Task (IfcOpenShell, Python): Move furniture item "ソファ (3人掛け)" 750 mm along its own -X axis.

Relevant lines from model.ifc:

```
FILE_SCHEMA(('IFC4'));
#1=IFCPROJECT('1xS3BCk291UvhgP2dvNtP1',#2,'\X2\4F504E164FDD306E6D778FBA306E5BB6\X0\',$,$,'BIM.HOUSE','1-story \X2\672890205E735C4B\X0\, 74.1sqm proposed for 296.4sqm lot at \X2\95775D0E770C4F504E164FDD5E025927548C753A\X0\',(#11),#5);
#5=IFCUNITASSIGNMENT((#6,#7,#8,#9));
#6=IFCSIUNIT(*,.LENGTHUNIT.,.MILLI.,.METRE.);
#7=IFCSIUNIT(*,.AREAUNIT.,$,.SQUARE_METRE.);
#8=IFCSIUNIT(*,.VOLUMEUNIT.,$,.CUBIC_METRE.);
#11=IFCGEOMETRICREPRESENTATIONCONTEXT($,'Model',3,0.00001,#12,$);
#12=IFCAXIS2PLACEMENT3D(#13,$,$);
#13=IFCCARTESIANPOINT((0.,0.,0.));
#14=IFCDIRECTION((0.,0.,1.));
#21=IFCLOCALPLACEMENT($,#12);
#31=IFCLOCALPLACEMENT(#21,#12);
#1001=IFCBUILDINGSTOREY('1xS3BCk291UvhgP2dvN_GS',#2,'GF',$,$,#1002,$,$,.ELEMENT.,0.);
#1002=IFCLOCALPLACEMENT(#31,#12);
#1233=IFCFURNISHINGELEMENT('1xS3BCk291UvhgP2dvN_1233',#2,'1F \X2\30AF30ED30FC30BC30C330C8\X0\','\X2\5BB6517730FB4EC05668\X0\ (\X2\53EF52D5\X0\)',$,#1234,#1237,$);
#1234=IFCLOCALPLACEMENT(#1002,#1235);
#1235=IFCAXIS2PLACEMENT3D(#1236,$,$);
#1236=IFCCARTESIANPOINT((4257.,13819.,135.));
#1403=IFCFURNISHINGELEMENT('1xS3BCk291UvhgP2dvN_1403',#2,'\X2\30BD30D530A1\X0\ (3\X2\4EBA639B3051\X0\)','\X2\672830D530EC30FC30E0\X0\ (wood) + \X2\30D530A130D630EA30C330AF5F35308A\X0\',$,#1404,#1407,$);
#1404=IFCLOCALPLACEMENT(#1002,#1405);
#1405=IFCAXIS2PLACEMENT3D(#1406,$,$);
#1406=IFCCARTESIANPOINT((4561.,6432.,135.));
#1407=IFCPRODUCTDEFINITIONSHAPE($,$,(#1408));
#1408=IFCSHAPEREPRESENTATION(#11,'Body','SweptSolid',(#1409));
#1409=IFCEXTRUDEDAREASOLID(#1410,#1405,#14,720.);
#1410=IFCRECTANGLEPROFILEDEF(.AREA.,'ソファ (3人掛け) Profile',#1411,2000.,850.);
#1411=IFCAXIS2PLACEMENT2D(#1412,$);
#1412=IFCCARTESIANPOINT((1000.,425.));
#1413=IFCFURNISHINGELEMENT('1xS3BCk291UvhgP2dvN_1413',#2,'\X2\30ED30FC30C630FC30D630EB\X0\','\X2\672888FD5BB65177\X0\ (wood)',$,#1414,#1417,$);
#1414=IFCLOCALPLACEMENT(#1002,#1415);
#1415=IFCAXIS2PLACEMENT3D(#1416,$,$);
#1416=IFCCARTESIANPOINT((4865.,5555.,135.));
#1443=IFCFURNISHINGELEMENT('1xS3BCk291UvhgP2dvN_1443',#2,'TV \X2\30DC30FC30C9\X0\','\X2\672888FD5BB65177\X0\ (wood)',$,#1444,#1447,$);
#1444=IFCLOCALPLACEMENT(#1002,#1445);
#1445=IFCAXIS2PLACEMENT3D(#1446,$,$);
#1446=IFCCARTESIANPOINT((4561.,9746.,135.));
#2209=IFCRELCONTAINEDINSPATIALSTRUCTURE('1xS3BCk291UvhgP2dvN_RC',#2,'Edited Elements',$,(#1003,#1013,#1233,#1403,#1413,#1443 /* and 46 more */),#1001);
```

```python
import ifcopenshell
import ifcopenshell.api.geometry
import ifcopenshell.util.placement

model = ifcopenshell.open("model.ifc")

item = model.by_guid("1xS3BCk291UvhgP2dvN_1403")
matrix = ifcopenshell.util.placement.get_local_placement(item.ObjectPlacement)
matrix[:3, 3] -= matrix[:3, 0] * 750.0
ifcopenshell.api.geometry.edit_object_placement(model, product=item, matrix=matrix, is_si=False)

print(ifcopenshell.util.placement.get_local_placement(item.ObjectPlacement).round(3) + 0.0)

model.write("model_rev.ifc")
```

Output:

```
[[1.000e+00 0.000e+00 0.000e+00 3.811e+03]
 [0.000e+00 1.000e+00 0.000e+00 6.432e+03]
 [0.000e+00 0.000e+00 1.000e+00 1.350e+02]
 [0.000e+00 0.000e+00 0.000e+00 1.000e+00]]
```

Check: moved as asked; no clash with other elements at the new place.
